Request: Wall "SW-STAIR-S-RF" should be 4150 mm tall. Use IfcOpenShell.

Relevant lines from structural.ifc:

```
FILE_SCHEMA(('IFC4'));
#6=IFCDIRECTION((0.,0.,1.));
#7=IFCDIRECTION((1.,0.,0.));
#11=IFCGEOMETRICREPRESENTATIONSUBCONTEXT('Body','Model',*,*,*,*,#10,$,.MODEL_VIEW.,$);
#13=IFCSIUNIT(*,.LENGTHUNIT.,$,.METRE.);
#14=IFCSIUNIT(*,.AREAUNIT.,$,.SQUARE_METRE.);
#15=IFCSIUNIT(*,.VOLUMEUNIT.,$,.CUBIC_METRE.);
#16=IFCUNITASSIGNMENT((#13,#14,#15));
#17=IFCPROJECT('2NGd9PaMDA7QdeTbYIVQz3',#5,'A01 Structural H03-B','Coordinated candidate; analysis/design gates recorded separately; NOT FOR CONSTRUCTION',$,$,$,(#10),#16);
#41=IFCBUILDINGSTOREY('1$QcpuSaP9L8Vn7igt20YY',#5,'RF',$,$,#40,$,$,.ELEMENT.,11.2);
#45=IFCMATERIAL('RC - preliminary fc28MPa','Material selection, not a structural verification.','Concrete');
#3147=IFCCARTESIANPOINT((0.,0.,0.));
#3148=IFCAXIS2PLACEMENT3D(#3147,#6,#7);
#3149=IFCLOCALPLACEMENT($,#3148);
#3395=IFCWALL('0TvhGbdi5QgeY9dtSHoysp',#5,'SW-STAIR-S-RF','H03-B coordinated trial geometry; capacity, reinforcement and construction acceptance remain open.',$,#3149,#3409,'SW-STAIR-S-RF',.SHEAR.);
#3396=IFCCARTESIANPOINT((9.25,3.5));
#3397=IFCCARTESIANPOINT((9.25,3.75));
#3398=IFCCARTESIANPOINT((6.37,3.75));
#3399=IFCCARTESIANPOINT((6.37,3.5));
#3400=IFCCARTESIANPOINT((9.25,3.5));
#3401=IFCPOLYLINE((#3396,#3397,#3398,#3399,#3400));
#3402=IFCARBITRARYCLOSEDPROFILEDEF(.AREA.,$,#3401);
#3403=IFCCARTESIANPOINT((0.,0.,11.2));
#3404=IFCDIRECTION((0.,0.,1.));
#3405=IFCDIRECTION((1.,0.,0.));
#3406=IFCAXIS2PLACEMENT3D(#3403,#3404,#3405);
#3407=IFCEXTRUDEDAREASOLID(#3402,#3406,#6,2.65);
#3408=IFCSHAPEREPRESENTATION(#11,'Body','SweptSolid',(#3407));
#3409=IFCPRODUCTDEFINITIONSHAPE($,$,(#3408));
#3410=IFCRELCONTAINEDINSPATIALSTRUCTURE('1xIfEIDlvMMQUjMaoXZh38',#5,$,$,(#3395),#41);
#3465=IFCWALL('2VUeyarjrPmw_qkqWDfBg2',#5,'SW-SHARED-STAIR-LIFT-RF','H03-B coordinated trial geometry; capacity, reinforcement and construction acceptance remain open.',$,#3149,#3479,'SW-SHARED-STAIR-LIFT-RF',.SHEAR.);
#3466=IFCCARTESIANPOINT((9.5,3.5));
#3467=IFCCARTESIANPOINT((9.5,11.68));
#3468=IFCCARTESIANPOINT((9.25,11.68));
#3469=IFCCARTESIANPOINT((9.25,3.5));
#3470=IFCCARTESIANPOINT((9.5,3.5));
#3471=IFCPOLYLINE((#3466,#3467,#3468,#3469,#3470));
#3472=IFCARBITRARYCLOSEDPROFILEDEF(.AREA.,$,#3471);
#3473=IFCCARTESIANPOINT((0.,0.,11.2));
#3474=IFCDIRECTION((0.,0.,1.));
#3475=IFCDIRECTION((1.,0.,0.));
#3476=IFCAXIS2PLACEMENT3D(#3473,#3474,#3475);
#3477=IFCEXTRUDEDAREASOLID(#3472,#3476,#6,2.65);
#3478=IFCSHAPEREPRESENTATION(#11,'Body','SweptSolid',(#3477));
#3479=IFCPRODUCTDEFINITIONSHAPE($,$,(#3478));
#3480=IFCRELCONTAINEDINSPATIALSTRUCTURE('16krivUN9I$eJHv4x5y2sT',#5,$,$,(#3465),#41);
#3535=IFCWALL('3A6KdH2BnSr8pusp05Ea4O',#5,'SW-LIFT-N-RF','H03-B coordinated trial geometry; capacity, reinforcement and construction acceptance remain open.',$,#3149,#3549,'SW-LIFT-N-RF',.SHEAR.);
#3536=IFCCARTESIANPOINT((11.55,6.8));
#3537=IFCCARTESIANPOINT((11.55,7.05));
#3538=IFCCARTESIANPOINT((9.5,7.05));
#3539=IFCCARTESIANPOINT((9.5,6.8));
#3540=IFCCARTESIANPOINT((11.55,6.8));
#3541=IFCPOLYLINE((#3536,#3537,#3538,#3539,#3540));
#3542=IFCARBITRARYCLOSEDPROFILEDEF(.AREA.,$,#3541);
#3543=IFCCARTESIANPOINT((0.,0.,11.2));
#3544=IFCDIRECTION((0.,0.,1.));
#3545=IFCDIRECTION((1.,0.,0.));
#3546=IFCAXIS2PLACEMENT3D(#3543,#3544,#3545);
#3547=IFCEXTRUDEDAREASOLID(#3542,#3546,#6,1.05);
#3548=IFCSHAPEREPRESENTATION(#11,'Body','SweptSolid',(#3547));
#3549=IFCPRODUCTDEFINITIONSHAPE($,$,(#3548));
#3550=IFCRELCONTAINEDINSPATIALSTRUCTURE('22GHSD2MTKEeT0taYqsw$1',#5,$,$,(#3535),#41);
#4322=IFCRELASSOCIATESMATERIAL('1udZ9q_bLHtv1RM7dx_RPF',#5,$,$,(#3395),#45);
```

```python
import ifcopenshell
import ifcopenshell.geom
import ifcopenshell.util.representation
import ifcopenshell.util.shape
import ifcopenshell.util.unit

model = ifcopenshell.open("structural.ifc")
unit_scale = ifcopenshell.util.unit.calculate_unit_scale(model)
settings = ifcopenshell.geom.settings()


def volume(element):
    """Net volume in cubic metres, openings subtracted."""
    shape = ifcopenshell.geom.create_shape(settings, element)
    return ifcopenshell.util.shape.get_volume(shape.geometry)


wall = model.by_guid("0TvhGbdi5QgeY9dtSHoysp")
before = volume(wall)

body = ifcopenshell.util.representation.get_representation(wall, "Model", "Body")
solid = body.Items[0]
old_height = solid.Depth
solid.Depth = 4.15 / unit_scale
after = volume(wall)

print(f"height {old_height:g} -> {solid.Depth:g}, volume {before:.3f} -> {after:.3f} m3")

model.write("structural_edited.ifc")
```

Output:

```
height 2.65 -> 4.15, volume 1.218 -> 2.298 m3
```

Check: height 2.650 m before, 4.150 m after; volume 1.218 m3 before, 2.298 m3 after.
